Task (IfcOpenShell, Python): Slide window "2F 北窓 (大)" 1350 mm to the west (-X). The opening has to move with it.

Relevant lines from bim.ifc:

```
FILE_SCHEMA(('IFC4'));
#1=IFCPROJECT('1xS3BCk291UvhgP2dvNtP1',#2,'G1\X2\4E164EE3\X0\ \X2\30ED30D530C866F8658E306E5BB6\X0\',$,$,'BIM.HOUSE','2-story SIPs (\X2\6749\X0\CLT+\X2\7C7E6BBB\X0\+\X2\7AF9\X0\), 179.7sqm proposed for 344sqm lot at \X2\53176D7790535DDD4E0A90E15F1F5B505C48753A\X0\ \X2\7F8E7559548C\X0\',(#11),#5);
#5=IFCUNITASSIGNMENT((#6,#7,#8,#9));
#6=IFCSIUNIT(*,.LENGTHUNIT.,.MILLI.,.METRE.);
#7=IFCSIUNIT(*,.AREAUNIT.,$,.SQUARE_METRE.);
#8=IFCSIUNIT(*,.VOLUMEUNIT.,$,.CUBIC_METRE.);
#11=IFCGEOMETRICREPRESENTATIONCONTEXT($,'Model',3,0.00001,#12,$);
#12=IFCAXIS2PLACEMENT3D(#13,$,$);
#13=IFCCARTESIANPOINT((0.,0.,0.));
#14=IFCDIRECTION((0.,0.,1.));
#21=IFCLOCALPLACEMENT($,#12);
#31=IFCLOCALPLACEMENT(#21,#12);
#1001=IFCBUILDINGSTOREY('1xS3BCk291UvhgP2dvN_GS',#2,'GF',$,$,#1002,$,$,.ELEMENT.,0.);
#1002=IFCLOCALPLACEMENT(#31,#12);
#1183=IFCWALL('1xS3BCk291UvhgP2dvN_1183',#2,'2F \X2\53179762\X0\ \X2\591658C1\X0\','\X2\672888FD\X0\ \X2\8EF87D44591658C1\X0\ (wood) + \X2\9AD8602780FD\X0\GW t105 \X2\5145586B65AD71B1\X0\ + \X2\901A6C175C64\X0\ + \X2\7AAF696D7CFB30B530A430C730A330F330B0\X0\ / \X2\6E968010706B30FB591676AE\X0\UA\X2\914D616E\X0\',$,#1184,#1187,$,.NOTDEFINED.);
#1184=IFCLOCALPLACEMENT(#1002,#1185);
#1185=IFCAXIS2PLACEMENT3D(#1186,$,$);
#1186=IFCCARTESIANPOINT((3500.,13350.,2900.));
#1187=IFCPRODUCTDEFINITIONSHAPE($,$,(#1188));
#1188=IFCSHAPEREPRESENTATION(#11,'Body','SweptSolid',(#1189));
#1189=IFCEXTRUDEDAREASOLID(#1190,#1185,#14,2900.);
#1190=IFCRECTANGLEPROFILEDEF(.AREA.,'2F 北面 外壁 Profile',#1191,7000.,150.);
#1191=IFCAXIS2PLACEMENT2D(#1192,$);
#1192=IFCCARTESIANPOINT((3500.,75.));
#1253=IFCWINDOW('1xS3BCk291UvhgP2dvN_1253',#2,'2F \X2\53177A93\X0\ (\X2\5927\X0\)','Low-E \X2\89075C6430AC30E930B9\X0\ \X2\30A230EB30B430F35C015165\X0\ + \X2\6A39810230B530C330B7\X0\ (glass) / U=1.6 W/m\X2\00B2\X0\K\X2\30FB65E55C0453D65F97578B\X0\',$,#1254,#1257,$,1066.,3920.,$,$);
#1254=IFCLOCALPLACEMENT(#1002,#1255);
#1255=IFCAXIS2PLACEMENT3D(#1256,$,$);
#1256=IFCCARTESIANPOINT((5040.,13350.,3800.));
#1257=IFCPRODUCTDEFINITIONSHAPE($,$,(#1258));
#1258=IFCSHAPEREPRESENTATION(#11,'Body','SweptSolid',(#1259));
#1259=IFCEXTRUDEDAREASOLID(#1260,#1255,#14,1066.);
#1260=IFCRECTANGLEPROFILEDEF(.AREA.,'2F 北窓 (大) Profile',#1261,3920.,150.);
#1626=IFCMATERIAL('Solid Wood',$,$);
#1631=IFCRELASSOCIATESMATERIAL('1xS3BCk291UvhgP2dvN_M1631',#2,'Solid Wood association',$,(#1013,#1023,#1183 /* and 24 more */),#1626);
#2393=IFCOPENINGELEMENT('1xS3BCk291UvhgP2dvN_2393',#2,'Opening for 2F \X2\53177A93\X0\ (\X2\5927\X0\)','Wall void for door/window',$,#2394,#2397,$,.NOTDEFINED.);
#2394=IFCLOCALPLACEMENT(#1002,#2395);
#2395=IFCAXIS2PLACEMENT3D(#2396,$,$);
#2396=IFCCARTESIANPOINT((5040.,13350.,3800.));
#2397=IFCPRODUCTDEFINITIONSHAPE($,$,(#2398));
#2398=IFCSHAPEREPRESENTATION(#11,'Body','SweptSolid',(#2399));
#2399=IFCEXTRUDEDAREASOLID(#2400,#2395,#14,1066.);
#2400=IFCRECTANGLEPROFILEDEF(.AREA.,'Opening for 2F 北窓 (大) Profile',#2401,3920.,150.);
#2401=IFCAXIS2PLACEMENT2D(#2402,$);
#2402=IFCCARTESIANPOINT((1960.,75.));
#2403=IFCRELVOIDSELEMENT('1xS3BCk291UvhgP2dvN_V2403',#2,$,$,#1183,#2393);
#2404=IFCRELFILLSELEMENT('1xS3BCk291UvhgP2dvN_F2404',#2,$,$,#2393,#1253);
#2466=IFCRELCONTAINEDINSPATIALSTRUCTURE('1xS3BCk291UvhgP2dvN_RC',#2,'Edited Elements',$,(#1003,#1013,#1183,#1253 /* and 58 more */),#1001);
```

```python
import ifcopenshell
import ifcopenshell.api.geometry
import ifcopenshell.util.placement
import ifcopenshell.util.unit

model = ifcopenshell.open("bim.ifc")
unit_scale = ifcopenshell.util.unit.calculate_unit_scale(model)

window = model.by_guid("1xS3BCk291UvhgP2dvN_1253")
opening = window.FillsVoids[0].RelatingOpeningElement
wall = opening.VoidsElements[0].RelatingBuildingElement

wall_matrix = ifcopenshell.util.placement.get_local_placement(wall.ObjectPlacement)
shift = wall_matrix[:3, 0] * -1.35 / unit_scale
before = ifcopenshell.util.placement.get_local_placement(window.ObjectPlacement)[:3, 3].copy()

# The window is not placed relative to its opening, so move both.
for product in (opening, window):
    matrix = ifcopenshell.util.placement.get_local_placement(product.ObjectPlacement)
    matrix[:3, 3] += shift
    ifcopenshell.api.geometry.edit_object_placement(model, product=product, matrix=matrix, is_si=False)

after = ifcopenshell.util.placement.get_local_placement(window.ObjectPlacement)[:3, 3]
print("window moved by", (after - before).round(3) + 0.0)

model.write("bim-out.ifc")
```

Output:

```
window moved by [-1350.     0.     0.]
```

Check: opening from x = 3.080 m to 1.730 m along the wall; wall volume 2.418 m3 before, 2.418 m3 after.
